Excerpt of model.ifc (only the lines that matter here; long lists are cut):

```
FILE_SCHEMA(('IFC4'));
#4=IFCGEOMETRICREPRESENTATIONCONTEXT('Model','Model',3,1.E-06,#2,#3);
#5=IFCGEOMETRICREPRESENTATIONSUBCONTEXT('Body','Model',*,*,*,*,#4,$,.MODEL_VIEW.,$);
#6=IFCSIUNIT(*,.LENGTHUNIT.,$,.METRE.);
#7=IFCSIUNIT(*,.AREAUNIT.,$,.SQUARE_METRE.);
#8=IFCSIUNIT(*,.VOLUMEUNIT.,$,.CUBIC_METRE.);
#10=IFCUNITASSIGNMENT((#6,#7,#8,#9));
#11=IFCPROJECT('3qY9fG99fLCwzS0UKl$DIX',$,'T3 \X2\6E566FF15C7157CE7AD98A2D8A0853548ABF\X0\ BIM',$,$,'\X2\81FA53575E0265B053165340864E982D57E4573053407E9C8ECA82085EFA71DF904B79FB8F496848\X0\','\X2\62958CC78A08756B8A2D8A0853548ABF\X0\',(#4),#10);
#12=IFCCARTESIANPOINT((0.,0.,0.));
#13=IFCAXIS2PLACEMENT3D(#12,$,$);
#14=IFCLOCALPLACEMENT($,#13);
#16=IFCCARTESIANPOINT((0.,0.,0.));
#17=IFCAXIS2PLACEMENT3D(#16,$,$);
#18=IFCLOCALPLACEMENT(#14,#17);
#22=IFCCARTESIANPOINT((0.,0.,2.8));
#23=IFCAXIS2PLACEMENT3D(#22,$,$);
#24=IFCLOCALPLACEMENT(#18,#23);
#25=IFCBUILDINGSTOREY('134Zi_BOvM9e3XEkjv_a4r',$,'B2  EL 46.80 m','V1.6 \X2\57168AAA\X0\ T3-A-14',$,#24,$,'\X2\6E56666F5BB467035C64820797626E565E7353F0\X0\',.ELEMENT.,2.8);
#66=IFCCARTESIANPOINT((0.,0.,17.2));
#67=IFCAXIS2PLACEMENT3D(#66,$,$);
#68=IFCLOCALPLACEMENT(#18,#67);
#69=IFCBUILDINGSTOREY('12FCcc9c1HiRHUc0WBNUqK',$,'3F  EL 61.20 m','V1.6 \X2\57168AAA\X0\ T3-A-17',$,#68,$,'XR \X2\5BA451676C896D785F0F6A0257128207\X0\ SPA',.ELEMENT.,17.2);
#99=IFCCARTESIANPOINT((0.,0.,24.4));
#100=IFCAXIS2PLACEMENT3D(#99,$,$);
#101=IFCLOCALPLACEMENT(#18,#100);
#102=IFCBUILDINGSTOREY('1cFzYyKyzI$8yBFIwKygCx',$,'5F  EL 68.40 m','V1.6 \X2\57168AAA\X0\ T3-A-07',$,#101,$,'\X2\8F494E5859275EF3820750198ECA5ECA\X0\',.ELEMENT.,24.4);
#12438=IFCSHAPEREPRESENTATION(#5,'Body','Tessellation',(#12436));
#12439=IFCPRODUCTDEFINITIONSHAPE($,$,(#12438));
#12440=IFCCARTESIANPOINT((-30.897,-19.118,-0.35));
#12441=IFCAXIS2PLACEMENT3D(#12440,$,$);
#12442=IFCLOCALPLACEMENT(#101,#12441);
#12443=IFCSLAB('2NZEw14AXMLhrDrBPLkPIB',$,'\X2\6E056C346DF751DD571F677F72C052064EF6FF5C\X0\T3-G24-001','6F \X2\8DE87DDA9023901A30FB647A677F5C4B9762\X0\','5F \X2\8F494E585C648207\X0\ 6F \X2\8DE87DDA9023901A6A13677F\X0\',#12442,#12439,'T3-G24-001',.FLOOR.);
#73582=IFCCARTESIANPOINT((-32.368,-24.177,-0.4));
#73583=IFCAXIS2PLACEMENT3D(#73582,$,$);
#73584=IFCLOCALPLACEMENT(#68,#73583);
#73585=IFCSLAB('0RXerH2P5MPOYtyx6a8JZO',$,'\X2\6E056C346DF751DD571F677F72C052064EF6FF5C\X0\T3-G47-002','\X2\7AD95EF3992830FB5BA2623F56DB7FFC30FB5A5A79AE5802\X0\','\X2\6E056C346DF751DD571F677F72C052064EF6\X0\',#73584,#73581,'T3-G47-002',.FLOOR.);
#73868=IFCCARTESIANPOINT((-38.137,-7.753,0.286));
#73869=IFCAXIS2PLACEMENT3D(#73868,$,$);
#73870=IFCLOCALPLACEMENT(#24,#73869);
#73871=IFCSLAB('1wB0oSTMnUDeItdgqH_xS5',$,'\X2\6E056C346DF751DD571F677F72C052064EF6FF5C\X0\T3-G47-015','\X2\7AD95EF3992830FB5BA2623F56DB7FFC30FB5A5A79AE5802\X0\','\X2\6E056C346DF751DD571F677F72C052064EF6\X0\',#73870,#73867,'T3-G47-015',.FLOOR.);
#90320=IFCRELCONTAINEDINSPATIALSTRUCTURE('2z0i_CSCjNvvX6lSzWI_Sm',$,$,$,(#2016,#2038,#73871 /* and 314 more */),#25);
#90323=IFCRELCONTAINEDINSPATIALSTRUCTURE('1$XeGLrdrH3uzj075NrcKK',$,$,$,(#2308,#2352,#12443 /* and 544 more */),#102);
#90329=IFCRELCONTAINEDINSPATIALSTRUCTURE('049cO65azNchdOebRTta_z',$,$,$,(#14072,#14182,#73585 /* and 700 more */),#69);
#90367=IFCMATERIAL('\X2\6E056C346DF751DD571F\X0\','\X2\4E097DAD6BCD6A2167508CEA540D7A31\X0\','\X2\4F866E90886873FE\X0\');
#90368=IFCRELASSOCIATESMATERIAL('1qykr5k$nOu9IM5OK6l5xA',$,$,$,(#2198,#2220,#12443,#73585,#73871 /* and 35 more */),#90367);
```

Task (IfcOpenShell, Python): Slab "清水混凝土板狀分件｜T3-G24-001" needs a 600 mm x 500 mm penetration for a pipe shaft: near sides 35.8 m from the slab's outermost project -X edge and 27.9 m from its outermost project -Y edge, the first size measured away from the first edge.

```python
import numpy as np
import ifcopenshell
import ifcopenshell.api.feature
import ifcopenshell.api.geometry
import ifcopenshell.api.root
import ifcopenshell.geom
import ifcopenshell.util.placement
import ifcopenshell.util.representation
import ifcopenshell.util.shape
import ifcopenshell.util.unit

model = ifcopenshell.open("model.ifc")
unit_scale = ifcopenshell.util.unit.calculate_unit_scale(model)
settings = ifcopenshell.geom.settings()


def volume(element):
    """Net volume in cubic metres, openings subtracted."""
    shape = ifcopenshell.geom.create_shape(settings, element)
    return ifcopenshell.util.shape.get_volume(shape.geometry)


slab = model.by_guid("2NZEw14AXMLhrDrBPLkPIB")
before = volume(slab)

# Extent in the slab's own axes, in metres. The edges named are its -X and -Y sides.
slab_shape = ifcopenshell.geom.create_shape(settings, slab)
vertices = ifcopenshell.util.shape.get_vertices(slab_shape.geometry)
x_min, y_min, bottom = vertices.min(axis=0)
top = vertices[:, 2].max()

opening = ifcopenshell.api.root.create_entity(model, ifc_class="IfcOpeningElement", name="Pipe shaft opening", predefined_type="OPENING")
context = ifcopenshell.util.representation.get_context(model, "Model", "Body", "MODEL_VIEW")
width, depth = 0.6, 0.5
outline = [(0.0, 0.0), (width, 0.0), (width, depth), (0.0, depth), (0.0, 0.0)]
# Overshoot both faces by 50 mm so the cut is clean.
shape = ifcopenshell.api.geometry.add_slab_representation(
    model, context=context, depth=top - bottom + 0.1, polyline=outline
)
ifcopenshell.api.geometry.assign_representation(model, product=opening, representation=shape)

matrix = ifcopenshell.util.placement.get_local_placement(slab.ObjectPlacement)
matrix[:, 3] = matrix @ np.append(np.array([x_min + 35.8, y_min + 27.9, bottom - 0.05]) / unit_scale, 1.0)
ifcopenshell.api.geometry.edit_object_placement(model, product=opening, matrix=matrix, is_si=False)
ifcopenshell.api.feature.add_feature(model, feature=opening, element=slab)

after = volume(slab)

print(f"slab volume {before:.3f} -> {after:.3f} m3")

model.write("model-out.ifc")
```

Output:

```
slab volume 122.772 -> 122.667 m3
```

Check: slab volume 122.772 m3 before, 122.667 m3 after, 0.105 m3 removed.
